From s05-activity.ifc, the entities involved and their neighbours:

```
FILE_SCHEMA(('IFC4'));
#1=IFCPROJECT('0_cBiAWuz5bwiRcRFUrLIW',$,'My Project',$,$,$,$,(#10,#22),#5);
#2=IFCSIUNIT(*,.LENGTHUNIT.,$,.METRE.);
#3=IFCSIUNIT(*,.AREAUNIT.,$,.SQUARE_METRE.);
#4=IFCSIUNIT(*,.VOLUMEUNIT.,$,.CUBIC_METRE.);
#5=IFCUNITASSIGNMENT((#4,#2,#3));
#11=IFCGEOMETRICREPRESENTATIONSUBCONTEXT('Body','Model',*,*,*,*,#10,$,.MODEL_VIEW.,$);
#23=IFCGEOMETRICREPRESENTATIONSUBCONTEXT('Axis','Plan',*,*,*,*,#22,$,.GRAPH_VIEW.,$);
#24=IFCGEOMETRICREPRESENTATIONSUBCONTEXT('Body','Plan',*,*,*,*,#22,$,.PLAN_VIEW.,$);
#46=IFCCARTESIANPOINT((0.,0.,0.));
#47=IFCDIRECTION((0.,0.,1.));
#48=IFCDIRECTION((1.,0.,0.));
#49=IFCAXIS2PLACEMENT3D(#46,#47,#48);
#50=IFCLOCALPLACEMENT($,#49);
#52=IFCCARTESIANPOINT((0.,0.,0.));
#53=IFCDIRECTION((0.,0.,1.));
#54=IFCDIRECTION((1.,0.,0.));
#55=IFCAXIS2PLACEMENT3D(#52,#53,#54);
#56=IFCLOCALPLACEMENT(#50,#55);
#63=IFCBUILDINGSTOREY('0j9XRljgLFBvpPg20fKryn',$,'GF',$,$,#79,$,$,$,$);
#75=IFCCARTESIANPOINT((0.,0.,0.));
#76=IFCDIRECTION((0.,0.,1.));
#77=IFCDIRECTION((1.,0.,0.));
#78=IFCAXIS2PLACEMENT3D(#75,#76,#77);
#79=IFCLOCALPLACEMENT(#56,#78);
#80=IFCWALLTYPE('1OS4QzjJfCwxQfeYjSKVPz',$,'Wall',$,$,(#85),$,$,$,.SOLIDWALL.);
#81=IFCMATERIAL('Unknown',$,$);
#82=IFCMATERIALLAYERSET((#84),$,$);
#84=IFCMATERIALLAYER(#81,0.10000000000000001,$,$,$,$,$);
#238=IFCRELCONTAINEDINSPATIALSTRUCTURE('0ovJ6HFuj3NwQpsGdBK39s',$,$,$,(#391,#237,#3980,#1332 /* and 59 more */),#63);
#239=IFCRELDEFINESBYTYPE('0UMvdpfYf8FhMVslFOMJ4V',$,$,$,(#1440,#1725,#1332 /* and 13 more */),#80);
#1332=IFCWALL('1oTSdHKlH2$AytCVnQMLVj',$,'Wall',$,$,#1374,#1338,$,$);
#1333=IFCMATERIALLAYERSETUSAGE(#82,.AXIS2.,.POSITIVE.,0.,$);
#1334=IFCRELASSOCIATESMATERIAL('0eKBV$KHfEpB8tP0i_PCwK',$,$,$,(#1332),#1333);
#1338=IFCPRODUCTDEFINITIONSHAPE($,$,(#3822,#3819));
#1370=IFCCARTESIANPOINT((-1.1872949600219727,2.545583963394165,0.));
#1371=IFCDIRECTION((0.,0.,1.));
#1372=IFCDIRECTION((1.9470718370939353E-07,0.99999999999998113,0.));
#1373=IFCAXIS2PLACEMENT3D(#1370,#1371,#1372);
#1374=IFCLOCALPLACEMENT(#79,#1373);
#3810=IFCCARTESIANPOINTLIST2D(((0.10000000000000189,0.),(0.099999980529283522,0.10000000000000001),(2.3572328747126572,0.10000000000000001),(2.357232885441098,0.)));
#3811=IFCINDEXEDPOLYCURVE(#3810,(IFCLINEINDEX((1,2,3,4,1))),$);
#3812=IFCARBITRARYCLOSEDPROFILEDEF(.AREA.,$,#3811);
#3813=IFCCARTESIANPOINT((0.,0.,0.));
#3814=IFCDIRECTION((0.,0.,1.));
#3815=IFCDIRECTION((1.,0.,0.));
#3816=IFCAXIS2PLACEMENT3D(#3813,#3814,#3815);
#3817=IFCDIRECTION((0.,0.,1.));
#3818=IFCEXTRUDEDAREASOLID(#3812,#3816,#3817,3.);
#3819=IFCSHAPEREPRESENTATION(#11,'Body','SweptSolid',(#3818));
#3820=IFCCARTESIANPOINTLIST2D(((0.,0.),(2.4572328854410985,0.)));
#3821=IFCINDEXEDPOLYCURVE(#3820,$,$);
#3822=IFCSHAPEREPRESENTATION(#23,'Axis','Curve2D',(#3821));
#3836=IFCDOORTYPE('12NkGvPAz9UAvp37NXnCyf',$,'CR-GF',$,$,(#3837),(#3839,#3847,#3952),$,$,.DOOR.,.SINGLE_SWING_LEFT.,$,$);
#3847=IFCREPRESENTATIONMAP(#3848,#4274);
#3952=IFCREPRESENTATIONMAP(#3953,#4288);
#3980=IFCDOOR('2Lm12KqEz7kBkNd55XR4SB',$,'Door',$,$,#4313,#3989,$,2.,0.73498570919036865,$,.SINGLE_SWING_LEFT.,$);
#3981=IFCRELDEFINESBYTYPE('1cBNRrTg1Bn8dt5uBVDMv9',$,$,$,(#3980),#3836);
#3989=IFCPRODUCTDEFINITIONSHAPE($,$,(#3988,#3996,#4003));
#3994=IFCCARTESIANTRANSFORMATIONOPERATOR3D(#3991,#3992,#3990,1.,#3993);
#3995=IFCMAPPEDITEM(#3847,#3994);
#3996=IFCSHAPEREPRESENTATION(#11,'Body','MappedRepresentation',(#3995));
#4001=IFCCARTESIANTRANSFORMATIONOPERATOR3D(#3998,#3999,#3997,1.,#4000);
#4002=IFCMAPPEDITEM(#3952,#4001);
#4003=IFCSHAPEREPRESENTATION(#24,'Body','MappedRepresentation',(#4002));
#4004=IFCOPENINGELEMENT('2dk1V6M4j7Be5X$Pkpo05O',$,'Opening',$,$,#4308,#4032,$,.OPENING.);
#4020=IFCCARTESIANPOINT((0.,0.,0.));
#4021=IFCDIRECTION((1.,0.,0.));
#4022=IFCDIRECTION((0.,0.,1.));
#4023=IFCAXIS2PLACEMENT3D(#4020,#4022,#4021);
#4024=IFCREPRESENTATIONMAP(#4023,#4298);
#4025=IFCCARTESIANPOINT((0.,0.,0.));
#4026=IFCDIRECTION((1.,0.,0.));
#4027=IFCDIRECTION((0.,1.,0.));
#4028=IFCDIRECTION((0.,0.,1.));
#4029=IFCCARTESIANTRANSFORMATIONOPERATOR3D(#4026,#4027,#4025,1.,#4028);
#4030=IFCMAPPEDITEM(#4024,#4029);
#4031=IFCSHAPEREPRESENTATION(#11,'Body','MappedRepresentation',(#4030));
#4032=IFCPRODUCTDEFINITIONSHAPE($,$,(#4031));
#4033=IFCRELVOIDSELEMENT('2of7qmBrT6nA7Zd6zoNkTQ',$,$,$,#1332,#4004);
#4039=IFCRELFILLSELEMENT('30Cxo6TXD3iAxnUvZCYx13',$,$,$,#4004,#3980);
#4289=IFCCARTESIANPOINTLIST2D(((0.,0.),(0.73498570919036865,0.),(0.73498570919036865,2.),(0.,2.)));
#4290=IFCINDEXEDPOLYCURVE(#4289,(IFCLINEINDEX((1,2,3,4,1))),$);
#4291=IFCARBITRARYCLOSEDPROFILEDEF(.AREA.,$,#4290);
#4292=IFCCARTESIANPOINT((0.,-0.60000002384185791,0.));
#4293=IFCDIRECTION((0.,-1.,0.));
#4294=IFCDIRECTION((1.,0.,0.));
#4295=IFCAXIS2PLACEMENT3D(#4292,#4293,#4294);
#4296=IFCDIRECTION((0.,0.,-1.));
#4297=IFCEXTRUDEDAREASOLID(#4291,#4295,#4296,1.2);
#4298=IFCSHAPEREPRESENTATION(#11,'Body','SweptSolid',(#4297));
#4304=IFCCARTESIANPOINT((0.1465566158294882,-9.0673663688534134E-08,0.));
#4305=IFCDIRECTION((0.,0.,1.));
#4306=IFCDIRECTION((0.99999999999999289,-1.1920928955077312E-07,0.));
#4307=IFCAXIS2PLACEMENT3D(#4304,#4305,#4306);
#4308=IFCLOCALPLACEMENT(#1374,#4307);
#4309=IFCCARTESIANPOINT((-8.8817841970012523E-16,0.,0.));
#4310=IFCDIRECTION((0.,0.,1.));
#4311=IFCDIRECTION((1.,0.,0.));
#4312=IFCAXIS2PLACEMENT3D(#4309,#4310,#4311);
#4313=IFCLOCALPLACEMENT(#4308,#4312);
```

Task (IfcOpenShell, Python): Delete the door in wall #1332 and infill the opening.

```python
import ifcopenshell
import ifcopenshell.api.feature
import ifcopenshell.api.root
import ifcopenshell.geom
import ifcopenshell.util.shape

model = ifcopenshell.open("s05-activity.ifc")
settings = ifcopenshell.geom.settings()


def volume(element):
    """Net volume in cubic metres, openings subtracted."""
    shape = ifcopenshell.geom.create_shape(settings, element)
    return ifcopenshell.util.shape.get_volume(shape.geometry)


door = model.by_guid("2Lm12KqEz7kBkNd55XR4SB")
opening = door.FillsVoids[0].RelatingOpeningElement
wall = opening.VoidsElements[0].RelatingBuildingElement
before = volume(wall)

ifcopenshell.api.root.remove_product(model, product=door)
ifcopenshell.api.feature.remove_feature(model, feature=opening)

after = volume(wall)

print(f"wall volume {before:.3f} -> {after:.3f} m3")

model.write("s05-activity-out.ifc")
```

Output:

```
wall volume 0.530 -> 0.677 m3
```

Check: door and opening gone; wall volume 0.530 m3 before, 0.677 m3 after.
